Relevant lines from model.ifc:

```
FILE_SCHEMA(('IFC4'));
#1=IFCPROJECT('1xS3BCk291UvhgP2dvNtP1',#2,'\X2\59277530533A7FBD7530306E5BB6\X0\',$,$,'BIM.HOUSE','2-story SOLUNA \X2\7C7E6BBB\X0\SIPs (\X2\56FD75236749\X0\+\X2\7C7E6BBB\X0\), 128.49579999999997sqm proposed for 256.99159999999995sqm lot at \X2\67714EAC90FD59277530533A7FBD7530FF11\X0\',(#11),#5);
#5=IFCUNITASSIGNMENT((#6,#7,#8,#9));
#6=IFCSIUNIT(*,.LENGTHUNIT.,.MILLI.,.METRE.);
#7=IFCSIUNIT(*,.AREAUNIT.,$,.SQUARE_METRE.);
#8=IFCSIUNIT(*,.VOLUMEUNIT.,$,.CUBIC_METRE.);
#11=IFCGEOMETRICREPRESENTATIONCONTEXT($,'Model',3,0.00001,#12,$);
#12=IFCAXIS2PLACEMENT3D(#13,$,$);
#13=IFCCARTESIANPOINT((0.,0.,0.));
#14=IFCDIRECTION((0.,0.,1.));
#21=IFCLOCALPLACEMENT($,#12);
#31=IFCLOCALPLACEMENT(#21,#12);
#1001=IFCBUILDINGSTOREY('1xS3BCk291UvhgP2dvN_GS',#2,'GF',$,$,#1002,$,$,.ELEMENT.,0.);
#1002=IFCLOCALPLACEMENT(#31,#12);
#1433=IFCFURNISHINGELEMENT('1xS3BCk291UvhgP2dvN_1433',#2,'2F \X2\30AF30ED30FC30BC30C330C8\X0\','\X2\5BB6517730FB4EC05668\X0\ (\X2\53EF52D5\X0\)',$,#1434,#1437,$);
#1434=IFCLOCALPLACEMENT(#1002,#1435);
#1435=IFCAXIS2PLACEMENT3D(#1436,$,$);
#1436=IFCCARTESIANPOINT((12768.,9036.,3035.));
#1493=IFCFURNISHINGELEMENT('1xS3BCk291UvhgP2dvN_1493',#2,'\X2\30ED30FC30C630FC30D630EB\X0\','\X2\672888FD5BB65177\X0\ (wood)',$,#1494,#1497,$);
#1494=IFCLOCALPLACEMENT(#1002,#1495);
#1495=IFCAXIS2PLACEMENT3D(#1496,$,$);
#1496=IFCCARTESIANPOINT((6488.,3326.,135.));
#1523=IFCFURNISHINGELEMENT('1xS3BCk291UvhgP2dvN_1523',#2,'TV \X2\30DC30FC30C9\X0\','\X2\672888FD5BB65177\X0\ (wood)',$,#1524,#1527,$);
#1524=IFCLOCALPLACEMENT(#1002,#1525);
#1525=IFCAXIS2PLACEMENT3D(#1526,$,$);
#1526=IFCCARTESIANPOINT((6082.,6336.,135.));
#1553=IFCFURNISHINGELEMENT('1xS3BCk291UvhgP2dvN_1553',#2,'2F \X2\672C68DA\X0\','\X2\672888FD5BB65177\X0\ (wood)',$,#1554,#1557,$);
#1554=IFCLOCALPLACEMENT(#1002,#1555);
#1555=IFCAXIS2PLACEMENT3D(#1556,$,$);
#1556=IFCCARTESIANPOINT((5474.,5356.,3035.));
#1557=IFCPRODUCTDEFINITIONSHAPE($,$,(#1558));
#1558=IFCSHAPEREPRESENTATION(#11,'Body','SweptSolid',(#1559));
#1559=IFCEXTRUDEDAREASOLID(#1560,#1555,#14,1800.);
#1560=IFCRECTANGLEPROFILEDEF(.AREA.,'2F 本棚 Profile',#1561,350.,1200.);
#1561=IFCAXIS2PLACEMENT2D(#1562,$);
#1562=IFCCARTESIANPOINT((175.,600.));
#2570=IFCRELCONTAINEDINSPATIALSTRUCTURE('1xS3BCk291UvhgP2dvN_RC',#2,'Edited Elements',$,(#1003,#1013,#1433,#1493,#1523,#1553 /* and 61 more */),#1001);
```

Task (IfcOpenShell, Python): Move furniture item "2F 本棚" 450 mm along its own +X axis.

```python
import ifcopenshell
import ifcopenshell.api.geometry
import ifcopenshell.util.placement
import ifcopenshell.util.unit

model = ifcopenshell.open("model.ifc")
unit_scale = ifcopenshell.util.unit.calculate_unit_scale(model)

item = model.by_id(1553)
matrix = ifcopenshell.util.placement.get_local_placement(item.ObjectPlacement)
matrix[:3, 3] += matrix[:3, 0] * 0.45 / unit_scale
ifcopenshell.api.geometry.edit_object_placement(model, product=item, matrix=matrix, is_si=False)

print(ifcopenshell.util.placement.get_local_placement(item.ObjectPlacement).round(3) + 0.0)

model.write("model-out.ifc")
```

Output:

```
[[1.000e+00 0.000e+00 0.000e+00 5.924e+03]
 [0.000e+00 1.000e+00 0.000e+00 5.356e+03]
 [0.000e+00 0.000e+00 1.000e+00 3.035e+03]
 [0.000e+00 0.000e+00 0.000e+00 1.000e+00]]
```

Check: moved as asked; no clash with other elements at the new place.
